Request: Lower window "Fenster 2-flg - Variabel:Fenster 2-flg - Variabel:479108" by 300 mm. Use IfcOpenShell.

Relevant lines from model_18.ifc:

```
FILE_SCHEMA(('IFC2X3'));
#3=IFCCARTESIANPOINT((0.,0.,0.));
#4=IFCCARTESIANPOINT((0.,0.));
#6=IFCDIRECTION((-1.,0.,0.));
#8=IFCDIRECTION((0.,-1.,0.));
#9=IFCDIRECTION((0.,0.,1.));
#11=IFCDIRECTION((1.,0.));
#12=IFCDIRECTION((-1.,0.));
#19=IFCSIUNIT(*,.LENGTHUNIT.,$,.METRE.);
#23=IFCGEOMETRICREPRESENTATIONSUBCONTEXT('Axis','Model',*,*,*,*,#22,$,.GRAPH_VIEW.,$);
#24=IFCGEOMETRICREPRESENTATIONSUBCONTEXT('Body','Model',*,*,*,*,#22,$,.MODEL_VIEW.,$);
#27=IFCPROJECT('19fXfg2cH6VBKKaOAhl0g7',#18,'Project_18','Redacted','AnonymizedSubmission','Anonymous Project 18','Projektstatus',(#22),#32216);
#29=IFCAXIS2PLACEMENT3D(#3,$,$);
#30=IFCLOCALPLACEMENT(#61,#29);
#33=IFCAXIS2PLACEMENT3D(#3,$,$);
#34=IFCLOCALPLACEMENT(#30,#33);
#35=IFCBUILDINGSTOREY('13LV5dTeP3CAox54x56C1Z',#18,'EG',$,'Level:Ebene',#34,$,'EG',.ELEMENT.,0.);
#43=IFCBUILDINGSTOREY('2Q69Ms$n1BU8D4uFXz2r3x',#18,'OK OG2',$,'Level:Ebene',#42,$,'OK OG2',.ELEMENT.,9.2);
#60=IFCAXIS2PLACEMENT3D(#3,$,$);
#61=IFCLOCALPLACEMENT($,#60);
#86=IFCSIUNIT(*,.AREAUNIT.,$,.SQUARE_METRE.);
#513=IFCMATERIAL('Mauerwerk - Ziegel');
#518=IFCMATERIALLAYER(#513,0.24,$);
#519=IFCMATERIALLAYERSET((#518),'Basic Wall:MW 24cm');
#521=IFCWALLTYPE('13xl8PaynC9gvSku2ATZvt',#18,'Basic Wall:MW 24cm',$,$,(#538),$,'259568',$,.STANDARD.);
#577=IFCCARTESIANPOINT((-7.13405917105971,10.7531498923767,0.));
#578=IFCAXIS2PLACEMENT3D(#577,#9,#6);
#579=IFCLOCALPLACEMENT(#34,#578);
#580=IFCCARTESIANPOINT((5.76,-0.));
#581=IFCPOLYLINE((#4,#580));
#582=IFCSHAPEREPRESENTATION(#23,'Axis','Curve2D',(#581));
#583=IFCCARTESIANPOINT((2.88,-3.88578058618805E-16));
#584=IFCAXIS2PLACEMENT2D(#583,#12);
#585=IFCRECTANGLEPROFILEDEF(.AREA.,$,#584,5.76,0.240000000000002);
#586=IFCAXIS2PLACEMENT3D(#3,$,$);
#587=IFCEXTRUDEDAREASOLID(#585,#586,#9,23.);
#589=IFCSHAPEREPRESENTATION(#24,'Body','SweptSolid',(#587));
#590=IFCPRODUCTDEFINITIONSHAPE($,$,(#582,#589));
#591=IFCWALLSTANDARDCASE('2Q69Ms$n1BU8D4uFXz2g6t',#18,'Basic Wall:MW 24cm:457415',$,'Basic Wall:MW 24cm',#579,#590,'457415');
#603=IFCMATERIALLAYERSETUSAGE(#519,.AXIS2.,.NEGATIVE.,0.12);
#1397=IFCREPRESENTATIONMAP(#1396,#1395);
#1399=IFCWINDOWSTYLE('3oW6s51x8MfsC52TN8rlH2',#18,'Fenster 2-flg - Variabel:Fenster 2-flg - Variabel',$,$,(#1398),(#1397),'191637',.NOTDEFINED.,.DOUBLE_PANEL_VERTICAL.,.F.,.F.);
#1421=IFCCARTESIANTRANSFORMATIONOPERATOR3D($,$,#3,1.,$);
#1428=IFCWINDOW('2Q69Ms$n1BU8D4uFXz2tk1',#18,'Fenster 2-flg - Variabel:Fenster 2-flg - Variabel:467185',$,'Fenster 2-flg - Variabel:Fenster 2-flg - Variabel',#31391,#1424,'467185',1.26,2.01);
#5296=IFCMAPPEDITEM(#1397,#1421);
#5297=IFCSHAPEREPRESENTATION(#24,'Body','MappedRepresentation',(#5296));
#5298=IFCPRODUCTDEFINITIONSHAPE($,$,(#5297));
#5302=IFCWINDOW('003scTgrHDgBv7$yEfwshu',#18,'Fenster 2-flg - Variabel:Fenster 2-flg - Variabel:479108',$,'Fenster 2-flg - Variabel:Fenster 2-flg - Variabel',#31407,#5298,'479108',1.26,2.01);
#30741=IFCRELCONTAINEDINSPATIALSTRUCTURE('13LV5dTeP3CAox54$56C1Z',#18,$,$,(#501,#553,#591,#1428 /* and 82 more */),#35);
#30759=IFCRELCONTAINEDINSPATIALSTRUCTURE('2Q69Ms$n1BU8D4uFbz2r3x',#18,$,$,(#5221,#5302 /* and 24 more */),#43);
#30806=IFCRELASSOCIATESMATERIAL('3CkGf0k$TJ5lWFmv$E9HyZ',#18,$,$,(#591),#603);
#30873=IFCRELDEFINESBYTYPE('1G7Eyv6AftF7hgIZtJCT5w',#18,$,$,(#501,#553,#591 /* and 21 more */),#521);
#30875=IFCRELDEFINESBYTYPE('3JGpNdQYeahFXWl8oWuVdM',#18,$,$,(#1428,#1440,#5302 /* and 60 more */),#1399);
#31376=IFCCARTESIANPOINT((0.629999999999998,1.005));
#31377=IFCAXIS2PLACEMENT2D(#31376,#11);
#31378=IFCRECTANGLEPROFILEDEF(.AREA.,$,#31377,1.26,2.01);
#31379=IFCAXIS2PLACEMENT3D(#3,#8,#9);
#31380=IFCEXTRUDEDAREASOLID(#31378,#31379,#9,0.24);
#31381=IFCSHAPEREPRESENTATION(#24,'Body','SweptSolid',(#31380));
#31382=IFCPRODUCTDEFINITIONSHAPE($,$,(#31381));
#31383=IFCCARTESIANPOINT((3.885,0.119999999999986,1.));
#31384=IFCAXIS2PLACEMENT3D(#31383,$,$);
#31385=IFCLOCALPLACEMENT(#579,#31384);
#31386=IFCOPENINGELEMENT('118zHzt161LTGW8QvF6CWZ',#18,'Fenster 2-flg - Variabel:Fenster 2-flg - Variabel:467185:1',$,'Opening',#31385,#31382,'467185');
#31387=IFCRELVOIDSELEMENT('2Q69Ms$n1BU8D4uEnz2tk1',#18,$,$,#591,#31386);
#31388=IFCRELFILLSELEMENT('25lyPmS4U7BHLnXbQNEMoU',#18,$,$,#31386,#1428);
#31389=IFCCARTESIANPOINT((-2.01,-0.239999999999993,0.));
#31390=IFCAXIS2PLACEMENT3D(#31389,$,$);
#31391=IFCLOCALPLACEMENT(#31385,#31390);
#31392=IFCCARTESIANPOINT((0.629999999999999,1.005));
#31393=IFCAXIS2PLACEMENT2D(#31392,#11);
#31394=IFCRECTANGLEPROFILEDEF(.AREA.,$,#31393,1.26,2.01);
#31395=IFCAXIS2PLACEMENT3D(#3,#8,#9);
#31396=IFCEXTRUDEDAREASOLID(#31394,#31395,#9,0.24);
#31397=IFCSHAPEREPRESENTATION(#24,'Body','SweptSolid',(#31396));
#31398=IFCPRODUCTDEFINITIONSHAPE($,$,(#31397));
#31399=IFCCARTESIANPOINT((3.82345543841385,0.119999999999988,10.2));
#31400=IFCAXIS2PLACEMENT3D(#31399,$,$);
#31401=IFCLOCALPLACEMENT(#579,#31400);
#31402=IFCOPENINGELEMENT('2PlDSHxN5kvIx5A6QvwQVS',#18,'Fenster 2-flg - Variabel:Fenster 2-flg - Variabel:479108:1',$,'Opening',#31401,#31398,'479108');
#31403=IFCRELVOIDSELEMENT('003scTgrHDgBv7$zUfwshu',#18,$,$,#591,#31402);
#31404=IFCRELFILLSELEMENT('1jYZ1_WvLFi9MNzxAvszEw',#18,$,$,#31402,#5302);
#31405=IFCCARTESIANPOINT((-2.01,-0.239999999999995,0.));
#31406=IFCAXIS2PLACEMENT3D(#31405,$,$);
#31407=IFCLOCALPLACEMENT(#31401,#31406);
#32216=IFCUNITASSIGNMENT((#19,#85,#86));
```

```python
import numpy as np
import ifcopenshell
import ifcopenshell.api.geometry
import ifcopenshell.util.placement
import ifcopenshell.util.unit

model = ifcopenshell.open("model_18.ifc")
unit_scale = ifcopenshell.util.unit.calculate_unit_scale(model)

window = model.by_id(5302)
opening = window.FillsVoids[0].RelatingOpeningElement
dz = -0.3

shift = np.array([0.0, 0.0, dz])
# The window is placed relative to its opening, so it follows when the opening moves.
matrix = ifcopenshell.util.placement.get_local_placement(opening.ObjectPlacement)
matrix[:3, 3] += shift
ifcopenshell.api.geometry.edit_object_placement(
    model, product=opening, matrix=matrix, is_si=False, should_transform_children=True
)

print(f"moved by {dz * unit_scale:+.3f} m")

model.write("model_18_rev.ifc")
```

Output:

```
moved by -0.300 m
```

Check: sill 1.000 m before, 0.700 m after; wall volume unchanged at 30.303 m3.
